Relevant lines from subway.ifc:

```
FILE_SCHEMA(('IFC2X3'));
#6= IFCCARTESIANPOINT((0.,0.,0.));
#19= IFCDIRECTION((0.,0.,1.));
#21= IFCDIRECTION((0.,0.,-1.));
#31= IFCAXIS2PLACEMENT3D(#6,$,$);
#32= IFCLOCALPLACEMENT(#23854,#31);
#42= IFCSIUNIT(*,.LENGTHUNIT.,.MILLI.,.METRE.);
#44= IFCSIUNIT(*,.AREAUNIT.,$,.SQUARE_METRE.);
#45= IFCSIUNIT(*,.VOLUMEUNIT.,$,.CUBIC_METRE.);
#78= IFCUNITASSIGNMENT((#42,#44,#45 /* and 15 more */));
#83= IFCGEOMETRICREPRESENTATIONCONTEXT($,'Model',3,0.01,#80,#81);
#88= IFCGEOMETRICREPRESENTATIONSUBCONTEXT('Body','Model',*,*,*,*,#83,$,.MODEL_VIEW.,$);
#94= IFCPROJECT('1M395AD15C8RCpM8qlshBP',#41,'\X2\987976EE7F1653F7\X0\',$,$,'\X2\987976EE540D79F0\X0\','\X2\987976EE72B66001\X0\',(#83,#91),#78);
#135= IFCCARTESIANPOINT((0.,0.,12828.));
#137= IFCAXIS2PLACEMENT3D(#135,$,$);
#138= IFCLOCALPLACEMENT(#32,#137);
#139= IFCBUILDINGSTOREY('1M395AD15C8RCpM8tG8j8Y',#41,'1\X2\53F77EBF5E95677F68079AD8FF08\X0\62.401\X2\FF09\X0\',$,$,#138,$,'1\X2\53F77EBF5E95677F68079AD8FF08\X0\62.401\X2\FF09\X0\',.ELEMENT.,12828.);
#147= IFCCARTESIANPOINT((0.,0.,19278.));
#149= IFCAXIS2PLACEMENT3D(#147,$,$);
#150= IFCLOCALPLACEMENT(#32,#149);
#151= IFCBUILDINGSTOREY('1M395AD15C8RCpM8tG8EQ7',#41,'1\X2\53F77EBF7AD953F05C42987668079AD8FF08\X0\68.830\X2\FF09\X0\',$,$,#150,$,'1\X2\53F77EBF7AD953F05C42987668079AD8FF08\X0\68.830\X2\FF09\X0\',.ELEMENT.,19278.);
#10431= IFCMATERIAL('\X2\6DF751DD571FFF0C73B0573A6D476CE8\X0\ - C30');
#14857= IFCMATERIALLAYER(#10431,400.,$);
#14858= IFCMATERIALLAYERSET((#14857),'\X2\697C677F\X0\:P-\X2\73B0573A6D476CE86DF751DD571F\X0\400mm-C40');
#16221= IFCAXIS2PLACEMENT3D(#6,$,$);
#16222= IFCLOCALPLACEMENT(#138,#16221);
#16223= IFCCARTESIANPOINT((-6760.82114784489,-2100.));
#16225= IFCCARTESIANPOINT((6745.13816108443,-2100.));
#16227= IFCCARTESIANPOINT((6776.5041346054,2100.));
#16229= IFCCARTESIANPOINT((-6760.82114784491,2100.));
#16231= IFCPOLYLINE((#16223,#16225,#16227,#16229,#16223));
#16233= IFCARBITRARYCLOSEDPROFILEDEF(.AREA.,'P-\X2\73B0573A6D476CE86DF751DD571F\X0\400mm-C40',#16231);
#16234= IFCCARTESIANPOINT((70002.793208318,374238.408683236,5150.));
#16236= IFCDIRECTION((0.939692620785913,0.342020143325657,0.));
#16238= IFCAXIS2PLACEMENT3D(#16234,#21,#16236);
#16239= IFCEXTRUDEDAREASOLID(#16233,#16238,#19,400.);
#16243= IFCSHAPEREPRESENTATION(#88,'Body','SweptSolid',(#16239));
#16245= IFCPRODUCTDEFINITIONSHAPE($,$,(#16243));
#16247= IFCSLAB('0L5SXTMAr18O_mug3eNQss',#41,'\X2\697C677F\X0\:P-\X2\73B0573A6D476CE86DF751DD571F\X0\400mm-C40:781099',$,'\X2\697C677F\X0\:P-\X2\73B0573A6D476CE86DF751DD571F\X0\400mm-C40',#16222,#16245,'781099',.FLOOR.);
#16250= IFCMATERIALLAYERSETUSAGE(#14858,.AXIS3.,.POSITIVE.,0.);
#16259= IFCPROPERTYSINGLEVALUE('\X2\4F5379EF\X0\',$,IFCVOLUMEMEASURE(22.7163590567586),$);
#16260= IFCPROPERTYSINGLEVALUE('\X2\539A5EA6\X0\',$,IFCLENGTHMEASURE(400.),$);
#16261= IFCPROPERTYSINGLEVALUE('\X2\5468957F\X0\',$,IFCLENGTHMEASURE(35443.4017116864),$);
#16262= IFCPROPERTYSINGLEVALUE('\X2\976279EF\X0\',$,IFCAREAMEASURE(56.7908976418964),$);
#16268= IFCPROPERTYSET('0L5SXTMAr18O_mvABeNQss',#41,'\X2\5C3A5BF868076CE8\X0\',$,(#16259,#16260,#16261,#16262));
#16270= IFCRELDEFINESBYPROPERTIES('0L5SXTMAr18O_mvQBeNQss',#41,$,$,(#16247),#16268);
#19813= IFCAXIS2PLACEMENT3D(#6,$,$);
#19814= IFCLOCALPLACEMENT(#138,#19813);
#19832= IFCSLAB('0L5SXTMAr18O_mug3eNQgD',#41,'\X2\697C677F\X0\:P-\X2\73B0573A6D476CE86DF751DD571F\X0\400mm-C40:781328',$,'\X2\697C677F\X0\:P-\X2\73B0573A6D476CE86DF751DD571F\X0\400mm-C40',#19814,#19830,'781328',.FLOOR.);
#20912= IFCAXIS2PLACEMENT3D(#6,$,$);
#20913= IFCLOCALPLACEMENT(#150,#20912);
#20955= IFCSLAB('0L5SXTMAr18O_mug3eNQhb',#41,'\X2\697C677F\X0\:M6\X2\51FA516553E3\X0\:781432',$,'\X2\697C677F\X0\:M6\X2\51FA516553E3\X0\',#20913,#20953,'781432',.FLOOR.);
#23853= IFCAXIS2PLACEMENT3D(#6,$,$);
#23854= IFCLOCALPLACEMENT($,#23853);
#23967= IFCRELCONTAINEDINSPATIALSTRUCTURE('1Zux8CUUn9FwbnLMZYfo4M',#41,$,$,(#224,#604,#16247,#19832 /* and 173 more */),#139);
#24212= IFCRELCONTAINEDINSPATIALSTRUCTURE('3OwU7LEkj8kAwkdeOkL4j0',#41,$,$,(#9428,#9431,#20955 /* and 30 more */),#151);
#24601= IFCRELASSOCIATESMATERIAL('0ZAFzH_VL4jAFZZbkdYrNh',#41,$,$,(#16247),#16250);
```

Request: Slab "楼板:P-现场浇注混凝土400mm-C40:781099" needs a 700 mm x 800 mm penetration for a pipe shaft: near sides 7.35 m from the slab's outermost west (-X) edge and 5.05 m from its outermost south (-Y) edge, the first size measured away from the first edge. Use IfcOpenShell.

```python
import numpy as np
import ifcopenshell
import ifcopenshell.api.feature
import ifcopenshell.api.geometry
import ifcopenshell.api.pset
import ifcopenshell.api.root
import ifcopenshell.geom
import ifcopenshell.util.element
import ifcopenshell.util.placement
import ifcopenshell.util.representation
import ifcopenshell.util.shape
import ifcopenshell.util.unit

model = ifcopenshell.open("subway.ifc")
unit_scale = ifcopenshell.util.unit.calculate_unit_scale(model)
area_scale = ifcopenshell.util.unit.calculate_unit_scale(model, "AREAUNIT")
volume_scale = ifcopenshell.util.unit.calculate_unit_scale(model, "VOLUMEUNIT")
settings = ifcopenshell.geom.settings()


def volume(element):
    """Net volume in cubic metres, openings subtracted."""
    shape = ifcopenshell.geom.create_shape(settings, element)
    return ifcopenshell.util.shape.get_volume(shape.geometry)


slab = model.by_id(16247)
before = volume(slab)

# Extent in the slab's own axes, in metres. The edges named are its -X and -Y sides.
slab_shape = ifcopenshell.geom.create_shape(settings, slab)
vertices = ifcopenshell.util.shape.get_vertices(slab_shape.geometry)
x_min, y_min, bottom = vertices.min(axis=0)
top = vertices[:, 2].max()

opening = ifcopenshell.api.root.create_entity(model, ifc_class="IfcOpeningElement", name="Pipe shaft opening")
context = ifcopenshell.util.representation.get_context(model, "Model", "Body", "MODEL_VIEW")
width, depth = 0.7, 0.8
outline = [(0.0, 0.0), (width, 0.0), (width, depth), (0.0, depth), (0.0, 0.0)]
# Overshoot both faces by 50 mm so the cut is clean.
shape = ifcopenshell.api.geometry.add_slab_representation(
    model, context=context, depth=top - bottom + 0.1, polyline=outline
)
ifcopenshell.api.geometry.assign_representation(model, product=opening, representation=shape)

matrix = ifcopenshell.util.placement.get_local_placement(slab.ObjectPlacement)
matrix[:, 3] = matrix @ np.append(np.array([x_min + 7.35, y_min + 5.05, bottom - 0.05]) / unit_scale, 1.0)
ifcopenshell.api.geometry.edit_object_placement(model, product=opening, matrix=matrix, is_si=False)
ifcopenshell.api.feature.add_feature(model, feature=opening, element=slab)

after = volume(slab)

# Update the slab's stored quantities.
pset = model.by_id(ifcopenshell.util.element.get_pset(slab, "尺寸标注", should_inherit=False)["id"])
ifcopenshell.api.pset.edit_pset(model, pset=pset, properties={
    "体积": model.create_entity("IfcVolumeMeasure", after / volume_scale),
    "面积": model.create_entity("IfcAreaMeasure", after / (top - bottom) / area_scale),
})

print(f"slab volume {before:.3f} -> {after:.3f} m3")

model.write("subway_updated.ifc")
```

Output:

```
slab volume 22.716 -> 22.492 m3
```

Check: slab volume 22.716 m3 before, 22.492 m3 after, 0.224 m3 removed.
